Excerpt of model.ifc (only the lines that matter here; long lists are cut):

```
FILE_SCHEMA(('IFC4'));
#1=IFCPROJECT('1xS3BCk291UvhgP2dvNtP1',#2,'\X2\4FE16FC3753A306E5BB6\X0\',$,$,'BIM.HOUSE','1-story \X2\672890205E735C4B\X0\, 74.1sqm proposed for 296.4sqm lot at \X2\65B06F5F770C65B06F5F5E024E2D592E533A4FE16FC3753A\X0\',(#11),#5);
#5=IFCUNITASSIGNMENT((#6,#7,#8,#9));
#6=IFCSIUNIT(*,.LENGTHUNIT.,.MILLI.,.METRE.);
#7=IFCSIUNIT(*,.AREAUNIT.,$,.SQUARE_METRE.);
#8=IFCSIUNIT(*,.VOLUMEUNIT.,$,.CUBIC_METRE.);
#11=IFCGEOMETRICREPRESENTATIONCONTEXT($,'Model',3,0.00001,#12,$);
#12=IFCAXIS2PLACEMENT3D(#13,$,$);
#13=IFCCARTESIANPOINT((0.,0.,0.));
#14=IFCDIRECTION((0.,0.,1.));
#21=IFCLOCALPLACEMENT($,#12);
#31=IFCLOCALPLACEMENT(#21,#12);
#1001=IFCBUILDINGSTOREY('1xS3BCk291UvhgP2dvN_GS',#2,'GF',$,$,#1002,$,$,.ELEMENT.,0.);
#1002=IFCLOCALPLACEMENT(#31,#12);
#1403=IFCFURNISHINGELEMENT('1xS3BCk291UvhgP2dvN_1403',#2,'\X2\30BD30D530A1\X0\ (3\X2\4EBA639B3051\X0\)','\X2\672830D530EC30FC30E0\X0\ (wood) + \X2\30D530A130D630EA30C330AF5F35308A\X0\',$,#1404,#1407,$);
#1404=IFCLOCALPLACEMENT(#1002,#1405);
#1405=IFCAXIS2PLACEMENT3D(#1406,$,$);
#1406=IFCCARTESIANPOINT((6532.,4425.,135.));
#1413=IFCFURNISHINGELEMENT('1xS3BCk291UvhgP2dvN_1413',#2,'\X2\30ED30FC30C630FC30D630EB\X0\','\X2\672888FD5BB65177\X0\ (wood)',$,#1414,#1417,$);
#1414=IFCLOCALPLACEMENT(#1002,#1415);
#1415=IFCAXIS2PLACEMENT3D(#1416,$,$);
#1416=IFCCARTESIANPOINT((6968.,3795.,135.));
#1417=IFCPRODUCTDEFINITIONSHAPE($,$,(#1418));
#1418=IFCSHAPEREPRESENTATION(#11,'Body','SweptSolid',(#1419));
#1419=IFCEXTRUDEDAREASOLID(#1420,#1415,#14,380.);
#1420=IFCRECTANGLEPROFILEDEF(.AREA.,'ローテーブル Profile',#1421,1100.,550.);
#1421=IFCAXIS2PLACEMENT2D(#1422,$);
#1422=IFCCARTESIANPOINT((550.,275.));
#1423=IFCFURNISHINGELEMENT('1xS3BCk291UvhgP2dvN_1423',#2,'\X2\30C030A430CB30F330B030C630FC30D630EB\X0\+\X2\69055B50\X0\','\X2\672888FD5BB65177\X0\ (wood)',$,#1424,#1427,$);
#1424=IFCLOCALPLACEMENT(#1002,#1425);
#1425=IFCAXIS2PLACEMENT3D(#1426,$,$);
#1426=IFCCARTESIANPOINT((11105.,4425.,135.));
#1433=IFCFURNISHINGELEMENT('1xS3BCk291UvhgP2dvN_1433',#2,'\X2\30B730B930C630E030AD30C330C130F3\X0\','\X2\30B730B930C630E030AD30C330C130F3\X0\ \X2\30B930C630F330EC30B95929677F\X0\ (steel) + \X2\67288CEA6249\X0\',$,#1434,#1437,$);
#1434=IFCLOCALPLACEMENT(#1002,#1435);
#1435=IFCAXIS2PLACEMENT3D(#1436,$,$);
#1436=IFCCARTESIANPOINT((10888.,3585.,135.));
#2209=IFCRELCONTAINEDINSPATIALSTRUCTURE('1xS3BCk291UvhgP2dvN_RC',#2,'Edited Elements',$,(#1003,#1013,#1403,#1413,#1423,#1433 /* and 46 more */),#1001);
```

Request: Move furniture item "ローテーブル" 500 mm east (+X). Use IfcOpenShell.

```python
import ifcopenshell
import ifcopenshell.api.geometry
import ifcopenshell.util.placement

model = ifcopenshell.open("model.ifc")

item = model.by_guid("1xS3BCk291UvhgP2dvN_1413")
matrix = ifcopenshell.util.placement.get_local_placement(item.ObjectPlacement)
matrix[0, 3] += 500.0
ifcopenshell.api.geometry.edit_object_placement(model, product=item, matrix=matrix, is_si=False)

print(ifcopenshell.util.placement.get_local_placement(item.ObjectPlacement).round(3) + 0.0)

model.write("model_v2.ifc")
```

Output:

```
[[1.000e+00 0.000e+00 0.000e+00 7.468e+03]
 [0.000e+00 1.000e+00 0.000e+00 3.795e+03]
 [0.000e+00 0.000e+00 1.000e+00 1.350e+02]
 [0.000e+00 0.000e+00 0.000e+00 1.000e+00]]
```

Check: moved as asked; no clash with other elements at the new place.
